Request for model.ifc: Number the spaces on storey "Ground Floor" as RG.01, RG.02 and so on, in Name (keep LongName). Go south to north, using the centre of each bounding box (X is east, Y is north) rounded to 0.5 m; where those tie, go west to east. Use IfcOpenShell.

First a look at what the model holds.

```python
import ifcopenshell
import ifcopenshell.util.element
import ifcopenshell.util.placement

model = ifcopenshell.open("model.ifc")
print(model.schema)
storey = next(s for s in model.by_type("IfcBuildingStorey") if s.Name == "Ground Floor")
spaces = [e for e in ifcopenshell.util.element.get_decomposition(storey) if e.is_a("IfcSpace")]
for e in sorted(spaces, key=lambda e: e.id()):
    origin = ifcopenshell.util.placement.get_local_placement(e.ObjectPlacement)[:3, 3]
    print(e.id(), e.Name, e.LongName, origin.round(2) + 0.0, sep=" | ")
```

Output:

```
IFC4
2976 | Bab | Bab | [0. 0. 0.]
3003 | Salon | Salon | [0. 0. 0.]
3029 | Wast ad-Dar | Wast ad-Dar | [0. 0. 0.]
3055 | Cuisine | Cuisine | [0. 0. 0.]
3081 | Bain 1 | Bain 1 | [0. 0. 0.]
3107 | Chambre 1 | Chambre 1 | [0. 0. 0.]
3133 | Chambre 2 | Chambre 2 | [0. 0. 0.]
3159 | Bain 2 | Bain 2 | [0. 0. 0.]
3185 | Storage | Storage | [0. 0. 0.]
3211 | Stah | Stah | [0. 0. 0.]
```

```python
import ifcopenshell
import ifcopenshell.geom
import ifcopenshell.util.element
import ifcopenshell.util.shape

model = ifcopenshell.open("model.ifc")
settings = ifcopenshell.geom.settings()
settings.set("use-world-coords", True)


def centre(element):
    shape = ifcopenshell.geom.create_shape(settings, element)
    return ifcopenshell.util.shape.get_bbox_centroid(shape.geometry)


storey = next(s for s in model.by_type("IfcBuildingStorey") if s.Name == "Ground Floor")
spaces = [e for e in ifcopenshell.util.element.get_decomposition(storey) if e.is_a("IfcSpace")]

# Insertion points can sit at a corner or the storey origin, so sort by the geometry (in metres).
centres = {e: centre(e) for e in spaces}
spaces.sort(key=lambda e: (round(centres[e][1] / 0.5), centres[e][0]))

for i, e in enumerate(spaces, start=1):
    number = f"RG.{i:02d}"
    e.Name = number
    print(e.id(), number)

model.write("model_rev.ifc")
```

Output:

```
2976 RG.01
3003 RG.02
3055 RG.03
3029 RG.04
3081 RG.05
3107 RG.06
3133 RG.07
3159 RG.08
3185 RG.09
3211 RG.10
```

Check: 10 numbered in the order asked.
